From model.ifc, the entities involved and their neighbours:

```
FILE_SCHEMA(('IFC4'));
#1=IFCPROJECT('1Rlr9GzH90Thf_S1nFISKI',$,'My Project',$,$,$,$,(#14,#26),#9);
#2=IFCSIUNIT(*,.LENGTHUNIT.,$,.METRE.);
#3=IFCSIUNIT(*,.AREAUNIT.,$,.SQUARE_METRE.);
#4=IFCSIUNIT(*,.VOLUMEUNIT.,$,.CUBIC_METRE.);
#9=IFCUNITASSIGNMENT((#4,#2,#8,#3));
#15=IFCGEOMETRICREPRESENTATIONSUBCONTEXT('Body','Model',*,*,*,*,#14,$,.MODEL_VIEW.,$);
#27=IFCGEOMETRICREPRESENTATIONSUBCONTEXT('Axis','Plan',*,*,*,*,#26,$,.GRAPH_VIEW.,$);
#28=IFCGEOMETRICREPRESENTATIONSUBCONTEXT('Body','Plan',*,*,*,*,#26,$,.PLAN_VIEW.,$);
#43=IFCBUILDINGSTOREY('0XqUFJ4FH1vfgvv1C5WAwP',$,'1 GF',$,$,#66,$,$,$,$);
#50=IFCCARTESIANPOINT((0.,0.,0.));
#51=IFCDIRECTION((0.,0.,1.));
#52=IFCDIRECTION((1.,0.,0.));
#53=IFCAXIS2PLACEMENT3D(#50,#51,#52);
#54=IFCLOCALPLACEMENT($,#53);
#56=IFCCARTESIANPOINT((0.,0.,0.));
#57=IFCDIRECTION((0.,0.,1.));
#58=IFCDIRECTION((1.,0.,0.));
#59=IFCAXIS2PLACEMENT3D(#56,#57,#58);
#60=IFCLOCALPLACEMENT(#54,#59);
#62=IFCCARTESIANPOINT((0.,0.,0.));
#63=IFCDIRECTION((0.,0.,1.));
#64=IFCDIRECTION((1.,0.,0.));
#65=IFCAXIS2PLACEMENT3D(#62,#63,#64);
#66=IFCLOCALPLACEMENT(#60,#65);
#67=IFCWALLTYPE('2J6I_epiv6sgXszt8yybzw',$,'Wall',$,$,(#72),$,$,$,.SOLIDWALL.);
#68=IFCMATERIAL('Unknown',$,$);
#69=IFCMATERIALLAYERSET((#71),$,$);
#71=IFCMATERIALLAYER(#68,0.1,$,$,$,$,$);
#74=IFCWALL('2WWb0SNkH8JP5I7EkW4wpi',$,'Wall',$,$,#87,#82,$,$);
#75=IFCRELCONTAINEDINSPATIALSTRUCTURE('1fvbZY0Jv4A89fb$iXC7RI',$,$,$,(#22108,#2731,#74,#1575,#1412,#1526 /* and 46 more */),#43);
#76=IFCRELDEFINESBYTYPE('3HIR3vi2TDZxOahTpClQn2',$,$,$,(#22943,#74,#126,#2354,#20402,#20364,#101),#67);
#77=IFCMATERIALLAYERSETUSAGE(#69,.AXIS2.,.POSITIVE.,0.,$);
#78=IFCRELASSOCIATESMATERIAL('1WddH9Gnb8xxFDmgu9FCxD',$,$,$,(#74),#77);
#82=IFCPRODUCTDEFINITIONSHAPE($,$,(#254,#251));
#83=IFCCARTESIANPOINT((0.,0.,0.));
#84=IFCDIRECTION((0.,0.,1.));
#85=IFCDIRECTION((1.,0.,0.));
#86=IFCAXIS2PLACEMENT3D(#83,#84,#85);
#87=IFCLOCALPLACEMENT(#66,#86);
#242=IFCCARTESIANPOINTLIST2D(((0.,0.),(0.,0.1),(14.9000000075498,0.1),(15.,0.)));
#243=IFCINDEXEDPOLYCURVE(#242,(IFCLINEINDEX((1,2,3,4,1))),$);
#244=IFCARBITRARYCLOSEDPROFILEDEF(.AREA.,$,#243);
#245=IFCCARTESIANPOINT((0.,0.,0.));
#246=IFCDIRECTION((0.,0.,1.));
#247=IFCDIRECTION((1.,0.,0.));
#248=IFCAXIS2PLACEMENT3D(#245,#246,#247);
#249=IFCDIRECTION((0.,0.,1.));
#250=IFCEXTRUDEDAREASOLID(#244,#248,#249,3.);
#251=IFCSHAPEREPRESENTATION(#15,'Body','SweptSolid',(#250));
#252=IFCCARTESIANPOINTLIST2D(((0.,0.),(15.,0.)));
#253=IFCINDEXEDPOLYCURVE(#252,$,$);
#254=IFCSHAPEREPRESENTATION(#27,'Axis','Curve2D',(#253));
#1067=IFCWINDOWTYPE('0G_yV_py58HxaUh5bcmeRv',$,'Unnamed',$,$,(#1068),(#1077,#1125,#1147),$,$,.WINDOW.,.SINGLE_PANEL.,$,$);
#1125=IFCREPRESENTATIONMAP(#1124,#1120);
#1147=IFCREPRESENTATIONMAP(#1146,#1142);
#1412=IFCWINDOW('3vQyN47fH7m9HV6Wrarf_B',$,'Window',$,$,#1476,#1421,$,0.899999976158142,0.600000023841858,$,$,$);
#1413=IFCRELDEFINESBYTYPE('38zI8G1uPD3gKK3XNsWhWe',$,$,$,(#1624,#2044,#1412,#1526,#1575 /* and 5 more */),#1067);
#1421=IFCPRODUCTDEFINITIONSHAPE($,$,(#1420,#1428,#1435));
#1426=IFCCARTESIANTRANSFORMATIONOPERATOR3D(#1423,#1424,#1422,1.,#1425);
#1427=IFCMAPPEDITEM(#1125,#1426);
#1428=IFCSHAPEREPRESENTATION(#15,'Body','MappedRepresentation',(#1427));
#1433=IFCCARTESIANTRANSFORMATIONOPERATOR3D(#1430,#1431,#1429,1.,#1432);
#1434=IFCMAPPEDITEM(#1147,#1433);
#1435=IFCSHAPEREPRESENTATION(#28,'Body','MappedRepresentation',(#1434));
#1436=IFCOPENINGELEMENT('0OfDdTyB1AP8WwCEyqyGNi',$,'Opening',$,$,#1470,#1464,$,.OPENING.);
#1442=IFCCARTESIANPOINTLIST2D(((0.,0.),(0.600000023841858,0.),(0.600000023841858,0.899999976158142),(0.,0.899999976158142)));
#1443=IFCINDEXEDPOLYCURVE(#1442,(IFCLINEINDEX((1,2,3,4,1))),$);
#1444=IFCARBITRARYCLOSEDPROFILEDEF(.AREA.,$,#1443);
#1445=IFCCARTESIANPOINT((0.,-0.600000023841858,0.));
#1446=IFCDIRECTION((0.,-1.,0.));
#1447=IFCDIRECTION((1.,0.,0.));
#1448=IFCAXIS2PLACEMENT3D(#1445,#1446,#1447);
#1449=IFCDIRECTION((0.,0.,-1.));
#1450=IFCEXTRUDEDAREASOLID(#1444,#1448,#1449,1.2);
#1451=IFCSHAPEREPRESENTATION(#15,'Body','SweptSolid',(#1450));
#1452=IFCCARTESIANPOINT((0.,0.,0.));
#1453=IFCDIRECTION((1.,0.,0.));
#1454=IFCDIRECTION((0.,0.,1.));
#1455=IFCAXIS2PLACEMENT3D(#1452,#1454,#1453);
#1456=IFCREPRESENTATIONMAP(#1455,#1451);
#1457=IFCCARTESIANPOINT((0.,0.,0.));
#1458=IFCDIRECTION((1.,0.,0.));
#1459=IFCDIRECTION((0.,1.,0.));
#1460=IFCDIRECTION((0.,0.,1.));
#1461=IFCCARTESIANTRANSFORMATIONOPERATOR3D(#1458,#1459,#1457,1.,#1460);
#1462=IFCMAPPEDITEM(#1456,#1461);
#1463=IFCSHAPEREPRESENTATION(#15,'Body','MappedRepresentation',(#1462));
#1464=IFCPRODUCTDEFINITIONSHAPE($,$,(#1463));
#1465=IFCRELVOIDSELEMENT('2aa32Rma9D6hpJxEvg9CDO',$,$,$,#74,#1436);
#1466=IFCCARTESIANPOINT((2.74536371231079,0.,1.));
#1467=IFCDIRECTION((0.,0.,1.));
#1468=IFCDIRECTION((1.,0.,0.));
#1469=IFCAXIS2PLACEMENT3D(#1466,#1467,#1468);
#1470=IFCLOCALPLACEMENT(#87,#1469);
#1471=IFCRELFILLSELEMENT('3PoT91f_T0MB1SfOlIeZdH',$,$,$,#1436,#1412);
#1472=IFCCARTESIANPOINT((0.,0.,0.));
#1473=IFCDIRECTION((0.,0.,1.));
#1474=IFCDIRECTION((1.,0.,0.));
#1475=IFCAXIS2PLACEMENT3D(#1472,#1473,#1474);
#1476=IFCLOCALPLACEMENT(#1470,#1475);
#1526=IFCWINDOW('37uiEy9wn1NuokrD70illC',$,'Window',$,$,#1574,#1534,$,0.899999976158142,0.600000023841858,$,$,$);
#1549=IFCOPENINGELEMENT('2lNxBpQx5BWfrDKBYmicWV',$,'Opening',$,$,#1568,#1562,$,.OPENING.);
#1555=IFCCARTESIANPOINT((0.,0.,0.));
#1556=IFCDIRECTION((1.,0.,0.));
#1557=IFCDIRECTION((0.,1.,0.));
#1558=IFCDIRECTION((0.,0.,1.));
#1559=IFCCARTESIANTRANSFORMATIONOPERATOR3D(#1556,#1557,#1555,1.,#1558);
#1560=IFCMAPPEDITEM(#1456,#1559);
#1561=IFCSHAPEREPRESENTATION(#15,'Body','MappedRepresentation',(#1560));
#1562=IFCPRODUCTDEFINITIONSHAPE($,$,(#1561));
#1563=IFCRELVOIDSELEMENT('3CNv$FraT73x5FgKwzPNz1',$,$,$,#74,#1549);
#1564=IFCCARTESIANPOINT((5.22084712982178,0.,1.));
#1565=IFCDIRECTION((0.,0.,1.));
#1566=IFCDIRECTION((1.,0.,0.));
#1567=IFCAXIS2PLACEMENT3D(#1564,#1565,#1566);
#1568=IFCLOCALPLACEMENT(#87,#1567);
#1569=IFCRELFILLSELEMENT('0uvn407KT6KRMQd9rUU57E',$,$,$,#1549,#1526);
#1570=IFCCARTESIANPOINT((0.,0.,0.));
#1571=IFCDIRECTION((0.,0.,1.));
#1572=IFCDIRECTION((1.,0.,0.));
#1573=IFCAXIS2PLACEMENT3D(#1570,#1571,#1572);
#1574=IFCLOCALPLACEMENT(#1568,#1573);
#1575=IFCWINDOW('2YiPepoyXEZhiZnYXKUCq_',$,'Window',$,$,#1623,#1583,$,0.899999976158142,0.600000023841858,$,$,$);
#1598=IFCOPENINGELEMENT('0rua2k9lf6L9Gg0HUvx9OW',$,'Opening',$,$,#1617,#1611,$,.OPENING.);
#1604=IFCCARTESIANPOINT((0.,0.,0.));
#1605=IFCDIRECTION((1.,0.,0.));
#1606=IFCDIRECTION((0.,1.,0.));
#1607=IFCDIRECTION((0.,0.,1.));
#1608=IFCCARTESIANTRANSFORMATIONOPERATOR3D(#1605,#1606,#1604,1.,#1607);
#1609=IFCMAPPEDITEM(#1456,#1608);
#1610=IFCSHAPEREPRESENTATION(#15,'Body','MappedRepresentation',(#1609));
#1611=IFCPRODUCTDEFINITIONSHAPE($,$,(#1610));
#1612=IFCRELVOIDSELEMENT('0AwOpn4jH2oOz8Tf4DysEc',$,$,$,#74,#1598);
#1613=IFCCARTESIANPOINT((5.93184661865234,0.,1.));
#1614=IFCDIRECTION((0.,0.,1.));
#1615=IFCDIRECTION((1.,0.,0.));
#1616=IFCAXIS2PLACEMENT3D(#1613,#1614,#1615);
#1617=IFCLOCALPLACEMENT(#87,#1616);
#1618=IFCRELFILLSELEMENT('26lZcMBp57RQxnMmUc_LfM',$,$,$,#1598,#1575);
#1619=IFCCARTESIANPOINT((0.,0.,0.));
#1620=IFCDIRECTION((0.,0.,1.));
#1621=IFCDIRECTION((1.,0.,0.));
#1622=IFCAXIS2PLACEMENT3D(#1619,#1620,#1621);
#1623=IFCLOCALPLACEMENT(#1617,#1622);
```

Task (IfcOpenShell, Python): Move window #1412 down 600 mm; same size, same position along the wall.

```python
import numpy as np
import ifcopenshell
import ifcopenshell.api.geometry
import ifcopenshell.util.placement
import ifcopenshell.util.unit

model = ifcopenshell.open("model.ifc")
unit_scale = ifcopenshell.util.unit.calculate_unit_scale(model)

window = model.by_guid("3vQyN47fH7m9HV6Wrarf_B")
opening = window.FillsVoids[0].RelatingOpeningElement
dz = -0.6

shift = np.array([0.0, 0.0, dz])
# The window is placed relative to its opening, so it follows when the opening moves.
matrix = ifcopenshell.util.placement.get_local_placement(opening.ObjectPlacement)
matrix[:3, 3] += shift
ifcopenshell.api.geometry.edit_object_placement(
    model, product=opening, matrix=matrix, is_si=False, should_transform_children=True
)

print(f"moved by {dz * unit_scale:+.3f} m")

model.write("model_updated.ifc")
```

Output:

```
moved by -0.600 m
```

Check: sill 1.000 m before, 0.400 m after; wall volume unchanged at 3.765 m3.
